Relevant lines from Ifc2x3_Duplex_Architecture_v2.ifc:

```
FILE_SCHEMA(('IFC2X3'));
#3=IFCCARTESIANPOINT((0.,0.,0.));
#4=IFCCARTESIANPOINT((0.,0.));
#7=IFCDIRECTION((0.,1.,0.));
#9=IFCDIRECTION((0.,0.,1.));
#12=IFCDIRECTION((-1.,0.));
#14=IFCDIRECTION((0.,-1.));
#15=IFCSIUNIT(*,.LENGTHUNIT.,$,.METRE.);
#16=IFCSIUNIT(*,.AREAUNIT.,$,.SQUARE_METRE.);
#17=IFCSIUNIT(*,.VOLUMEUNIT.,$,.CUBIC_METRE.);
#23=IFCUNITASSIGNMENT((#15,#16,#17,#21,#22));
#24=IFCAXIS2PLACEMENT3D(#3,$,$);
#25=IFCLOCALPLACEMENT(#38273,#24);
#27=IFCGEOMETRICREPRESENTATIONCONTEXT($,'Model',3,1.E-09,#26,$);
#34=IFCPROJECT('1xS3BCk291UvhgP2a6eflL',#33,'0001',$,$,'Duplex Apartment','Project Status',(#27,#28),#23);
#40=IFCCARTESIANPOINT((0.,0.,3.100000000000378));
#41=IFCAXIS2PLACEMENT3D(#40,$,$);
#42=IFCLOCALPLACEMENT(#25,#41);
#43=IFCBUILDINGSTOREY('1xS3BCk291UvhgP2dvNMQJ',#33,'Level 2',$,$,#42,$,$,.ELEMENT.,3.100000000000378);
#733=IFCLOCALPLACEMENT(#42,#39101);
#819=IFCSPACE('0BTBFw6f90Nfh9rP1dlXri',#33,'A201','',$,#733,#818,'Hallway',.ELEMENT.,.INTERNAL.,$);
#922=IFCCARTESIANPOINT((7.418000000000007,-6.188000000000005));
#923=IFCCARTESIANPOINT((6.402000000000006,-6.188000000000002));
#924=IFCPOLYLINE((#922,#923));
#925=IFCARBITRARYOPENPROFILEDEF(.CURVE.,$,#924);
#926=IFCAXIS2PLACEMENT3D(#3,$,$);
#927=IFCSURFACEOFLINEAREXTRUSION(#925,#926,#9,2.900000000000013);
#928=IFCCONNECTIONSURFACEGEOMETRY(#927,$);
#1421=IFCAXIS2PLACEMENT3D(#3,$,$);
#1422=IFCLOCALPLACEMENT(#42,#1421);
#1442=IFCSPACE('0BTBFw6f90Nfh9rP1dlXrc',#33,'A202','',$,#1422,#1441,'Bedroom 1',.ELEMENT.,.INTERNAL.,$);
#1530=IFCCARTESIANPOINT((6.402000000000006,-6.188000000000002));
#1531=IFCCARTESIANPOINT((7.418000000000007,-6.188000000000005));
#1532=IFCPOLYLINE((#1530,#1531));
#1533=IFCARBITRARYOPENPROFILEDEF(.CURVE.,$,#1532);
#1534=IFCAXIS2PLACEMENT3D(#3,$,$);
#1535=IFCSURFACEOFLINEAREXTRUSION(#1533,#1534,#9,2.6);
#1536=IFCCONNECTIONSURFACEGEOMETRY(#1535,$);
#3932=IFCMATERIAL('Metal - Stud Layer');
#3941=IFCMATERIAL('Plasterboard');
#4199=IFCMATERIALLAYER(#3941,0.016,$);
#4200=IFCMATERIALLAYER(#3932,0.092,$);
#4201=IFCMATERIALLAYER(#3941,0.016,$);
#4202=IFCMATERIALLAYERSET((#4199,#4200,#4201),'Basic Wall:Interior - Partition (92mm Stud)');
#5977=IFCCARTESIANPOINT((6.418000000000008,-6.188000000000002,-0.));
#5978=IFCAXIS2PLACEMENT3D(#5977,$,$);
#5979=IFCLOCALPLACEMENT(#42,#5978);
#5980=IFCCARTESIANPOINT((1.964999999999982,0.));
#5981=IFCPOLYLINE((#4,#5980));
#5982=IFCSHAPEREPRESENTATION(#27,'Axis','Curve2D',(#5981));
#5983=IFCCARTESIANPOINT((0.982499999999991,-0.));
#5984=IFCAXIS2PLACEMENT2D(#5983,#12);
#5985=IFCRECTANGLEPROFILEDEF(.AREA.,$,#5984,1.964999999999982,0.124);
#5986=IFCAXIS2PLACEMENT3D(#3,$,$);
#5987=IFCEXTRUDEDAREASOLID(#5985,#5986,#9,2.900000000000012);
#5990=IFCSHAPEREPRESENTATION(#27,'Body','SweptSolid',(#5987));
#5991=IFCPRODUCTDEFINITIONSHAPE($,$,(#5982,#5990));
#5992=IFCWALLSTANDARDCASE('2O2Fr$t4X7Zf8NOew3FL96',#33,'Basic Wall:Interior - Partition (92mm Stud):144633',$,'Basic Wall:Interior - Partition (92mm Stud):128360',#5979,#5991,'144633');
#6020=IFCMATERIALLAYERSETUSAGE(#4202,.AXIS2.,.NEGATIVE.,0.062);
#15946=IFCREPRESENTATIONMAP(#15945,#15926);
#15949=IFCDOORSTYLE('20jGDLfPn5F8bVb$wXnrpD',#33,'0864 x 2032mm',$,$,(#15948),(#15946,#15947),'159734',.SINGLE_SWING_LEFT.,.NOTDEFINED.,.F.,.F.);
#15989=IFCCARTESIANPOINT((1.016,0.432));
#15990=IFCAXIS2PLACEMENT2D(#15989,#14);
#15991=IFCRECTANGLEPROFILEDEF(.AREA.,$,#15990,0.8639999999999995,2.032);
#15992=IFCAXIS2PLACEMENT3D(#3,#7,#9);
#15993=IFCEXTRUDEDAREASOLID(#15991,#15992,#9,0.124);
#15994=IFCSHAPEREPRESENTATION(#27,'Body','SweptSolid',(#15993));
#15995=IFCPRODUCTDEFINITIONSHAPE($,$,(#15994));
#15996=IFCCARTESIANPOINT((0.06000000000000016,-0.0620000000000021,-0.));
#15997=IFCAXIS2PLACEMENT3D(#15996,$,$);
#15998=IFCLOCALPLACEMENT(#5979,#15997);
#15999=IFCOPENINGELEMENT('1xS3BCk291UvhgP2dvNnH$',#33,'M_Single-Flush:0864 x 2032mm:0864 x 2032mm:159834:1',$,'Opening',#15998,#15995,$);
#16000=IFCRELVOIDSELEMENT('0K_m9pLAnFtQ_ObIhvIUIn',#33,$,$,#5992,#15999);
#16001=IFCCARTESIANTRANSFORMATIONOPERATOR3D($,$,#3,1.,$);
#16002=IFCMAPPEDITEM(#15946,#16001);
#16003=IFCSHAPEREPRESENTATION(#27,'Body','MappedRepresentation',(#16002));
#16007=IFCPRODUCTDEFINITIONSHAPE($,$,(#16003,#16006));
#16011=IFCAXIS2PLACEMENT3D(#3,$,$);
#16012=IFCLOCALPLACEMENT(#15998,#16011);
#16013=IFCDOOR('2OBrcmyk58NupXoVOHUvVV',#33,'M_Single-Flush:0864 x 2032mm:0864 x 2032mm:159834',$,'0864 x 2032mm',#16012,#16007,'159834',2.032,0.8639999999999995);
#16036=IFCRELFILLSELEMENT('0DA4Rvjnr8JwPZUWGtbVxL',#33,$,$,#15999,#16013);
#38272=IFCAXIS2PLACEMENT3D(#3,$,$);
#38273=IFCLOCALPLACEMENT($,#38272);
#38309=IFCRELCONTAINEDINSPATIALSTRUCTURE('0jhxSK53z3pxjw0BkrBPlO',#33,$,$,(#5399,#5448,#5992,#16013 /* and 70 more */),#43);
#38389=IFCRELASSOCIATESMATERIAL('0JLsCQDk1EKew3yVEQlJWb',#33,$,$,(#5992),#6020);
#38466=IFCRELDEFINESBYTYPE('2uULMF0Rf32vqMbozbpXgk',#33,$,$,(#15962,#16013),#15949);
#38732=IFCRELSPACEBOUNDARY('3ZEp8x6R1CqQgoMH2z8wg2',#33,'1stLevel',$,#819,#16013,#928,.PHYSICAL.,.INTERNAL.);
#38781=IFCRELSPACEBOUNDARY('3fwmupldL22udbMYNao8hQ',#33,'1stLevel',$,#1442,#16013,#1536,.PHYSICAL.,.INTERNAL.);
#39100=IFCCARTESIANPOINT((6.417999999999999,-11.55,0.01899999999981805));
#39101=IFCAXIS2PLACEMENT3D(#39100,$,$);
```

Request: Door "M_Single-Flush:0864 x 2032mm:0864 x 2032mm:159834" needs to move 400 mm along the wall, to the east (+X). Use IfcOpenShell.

```python
import numpy as np
import ifcopenshell
import ifcopenshell.api.geometry
import ifcopenshell.util.placement

model = ifcopenshell.open("Ifc2x3_Duplex_Architecture_v2.ifc")

door = model.by_guid("2OBrcmyk58NupXoVOHUvVV")
opening = door.FillsVoids[0].RelatingOpeningElement
wall = opening.VoidsElements[0].RelatingBuildingElement

wall_matrix = ifcopenshell.util.placement.get_local_placement(wall.ObjectPlacement)
shift = wall_matrix[:3, 0] * 0.4
before = ifcopenshell.util.placement.get_local_placement(door.ObjectPlacement)[:3, 3].copy()

# The door is placed relative to its opening, so it follows when the opening moves.
matrix = ifcopenshell.util.placement.get_local_placement(opening.ObjectPlacement)
matrix[:3, 3] += shift
ifcopenshell.api.geometry.edit_object_placement(
    model, product=opening, matrix=matrix, is_si=False, should_transform_children=True
)

# Space boundary surfaces are stored in each space's coordinates; move them too.
for rel in door.ProvidesBoundaries:
    if not rel.ConnectionGeometry:
        continue
    surface = rel.ConnectionGeometry.SurfaceOnRelatingElement
    space_matrix = ifcopenshell.util.placement.get_local_placement(rel.RelatingSpace.ObjectPlacement)
    point = np.array(surface.Position.Location.Coordinates) + space_matrix[:3, :3].T @ shift
    surface.Position = model.createIfcAxis2Placement3D(
        model.createIfcCartesianPoint(point.tolist()), surface.Position.Axis, surface.Position.RefDirection
    )

after = ifcopenshell.util.placement.get_local_placement(door.ObjectPlacement)[:3, 3]
print("door moved by", (after - before).round(3) + 0.0)

model.write("Ifc2x3_Duplex_Architecture_v2_updated.ifc")
```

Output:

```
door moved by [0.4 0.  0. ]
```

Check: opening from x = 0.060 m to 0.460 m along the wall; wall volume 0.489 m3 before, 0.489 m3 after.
